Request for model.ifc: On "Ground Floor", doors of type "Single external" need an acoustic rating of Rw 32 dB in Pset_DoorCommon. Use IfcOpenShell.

First a look at what the model holds.

```python
import ifcopenshell
import ifcopenshell.util.element

model = ifcopenshell.open("model.ifc")
print(model.schema)
storey = next(s for s in model.by_type("IfcBuildingStorey") if s.Name == "Ground Floor")
doors = [e for e in ifcopenshell.util.element.get_decomposition(storey) if e.is_a("IfcDoor")]
seen = {}
for e in doors:
    element_type = ifcopenshell.util.element.get_type(e)
    key = (element_type.Name if element_type != e and element_type else None, ifcopenshell.util.element.get_pset(e, "Pset_DoorCommon", "AcousticRating"))
    seen[key] = seen.get(key, 0) + 1
for (name, value), count in sorted(seen.items(), key=str):
    print(count, "x", name, "|", value)
```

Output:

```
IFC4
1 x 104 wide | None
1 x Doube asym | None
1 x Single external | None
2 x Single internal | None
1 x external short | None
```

```python
import ifcopenshell
import ifcopenshell.api.pset
import ifcopenshell.util.element

model = ifcopenshell.open("model.ifc")

storey = next(s for s in model.by_type("IfcBuildingStorey") if s.Name == "Ground Floor")
doors = [e for e in ifcopenshell.util.element.get_decomposition(storey) if e.is_a("IfcDoor")]

count = 0
for e in doors:
    element_type = ifcopenshell.util.element.get_type(e)
    if element_type in (None, e) or element_type.Name != "Single external":
        continue
    # add_pset returns the element's existing set when there is one.
    pset = ifcopenshell.api.pset.add_pset(model, product=e, name="Pset_DoorCommon")
    ifcopenshell.api.pset.edit_pset(model, pset=pset, properties={"AcousticRating": "Rw 32 dB"})
    count += 1

print(count, "doors updated")

model.write("model_updated.ifc")
```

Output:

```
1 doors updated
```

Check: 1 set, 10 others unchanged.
